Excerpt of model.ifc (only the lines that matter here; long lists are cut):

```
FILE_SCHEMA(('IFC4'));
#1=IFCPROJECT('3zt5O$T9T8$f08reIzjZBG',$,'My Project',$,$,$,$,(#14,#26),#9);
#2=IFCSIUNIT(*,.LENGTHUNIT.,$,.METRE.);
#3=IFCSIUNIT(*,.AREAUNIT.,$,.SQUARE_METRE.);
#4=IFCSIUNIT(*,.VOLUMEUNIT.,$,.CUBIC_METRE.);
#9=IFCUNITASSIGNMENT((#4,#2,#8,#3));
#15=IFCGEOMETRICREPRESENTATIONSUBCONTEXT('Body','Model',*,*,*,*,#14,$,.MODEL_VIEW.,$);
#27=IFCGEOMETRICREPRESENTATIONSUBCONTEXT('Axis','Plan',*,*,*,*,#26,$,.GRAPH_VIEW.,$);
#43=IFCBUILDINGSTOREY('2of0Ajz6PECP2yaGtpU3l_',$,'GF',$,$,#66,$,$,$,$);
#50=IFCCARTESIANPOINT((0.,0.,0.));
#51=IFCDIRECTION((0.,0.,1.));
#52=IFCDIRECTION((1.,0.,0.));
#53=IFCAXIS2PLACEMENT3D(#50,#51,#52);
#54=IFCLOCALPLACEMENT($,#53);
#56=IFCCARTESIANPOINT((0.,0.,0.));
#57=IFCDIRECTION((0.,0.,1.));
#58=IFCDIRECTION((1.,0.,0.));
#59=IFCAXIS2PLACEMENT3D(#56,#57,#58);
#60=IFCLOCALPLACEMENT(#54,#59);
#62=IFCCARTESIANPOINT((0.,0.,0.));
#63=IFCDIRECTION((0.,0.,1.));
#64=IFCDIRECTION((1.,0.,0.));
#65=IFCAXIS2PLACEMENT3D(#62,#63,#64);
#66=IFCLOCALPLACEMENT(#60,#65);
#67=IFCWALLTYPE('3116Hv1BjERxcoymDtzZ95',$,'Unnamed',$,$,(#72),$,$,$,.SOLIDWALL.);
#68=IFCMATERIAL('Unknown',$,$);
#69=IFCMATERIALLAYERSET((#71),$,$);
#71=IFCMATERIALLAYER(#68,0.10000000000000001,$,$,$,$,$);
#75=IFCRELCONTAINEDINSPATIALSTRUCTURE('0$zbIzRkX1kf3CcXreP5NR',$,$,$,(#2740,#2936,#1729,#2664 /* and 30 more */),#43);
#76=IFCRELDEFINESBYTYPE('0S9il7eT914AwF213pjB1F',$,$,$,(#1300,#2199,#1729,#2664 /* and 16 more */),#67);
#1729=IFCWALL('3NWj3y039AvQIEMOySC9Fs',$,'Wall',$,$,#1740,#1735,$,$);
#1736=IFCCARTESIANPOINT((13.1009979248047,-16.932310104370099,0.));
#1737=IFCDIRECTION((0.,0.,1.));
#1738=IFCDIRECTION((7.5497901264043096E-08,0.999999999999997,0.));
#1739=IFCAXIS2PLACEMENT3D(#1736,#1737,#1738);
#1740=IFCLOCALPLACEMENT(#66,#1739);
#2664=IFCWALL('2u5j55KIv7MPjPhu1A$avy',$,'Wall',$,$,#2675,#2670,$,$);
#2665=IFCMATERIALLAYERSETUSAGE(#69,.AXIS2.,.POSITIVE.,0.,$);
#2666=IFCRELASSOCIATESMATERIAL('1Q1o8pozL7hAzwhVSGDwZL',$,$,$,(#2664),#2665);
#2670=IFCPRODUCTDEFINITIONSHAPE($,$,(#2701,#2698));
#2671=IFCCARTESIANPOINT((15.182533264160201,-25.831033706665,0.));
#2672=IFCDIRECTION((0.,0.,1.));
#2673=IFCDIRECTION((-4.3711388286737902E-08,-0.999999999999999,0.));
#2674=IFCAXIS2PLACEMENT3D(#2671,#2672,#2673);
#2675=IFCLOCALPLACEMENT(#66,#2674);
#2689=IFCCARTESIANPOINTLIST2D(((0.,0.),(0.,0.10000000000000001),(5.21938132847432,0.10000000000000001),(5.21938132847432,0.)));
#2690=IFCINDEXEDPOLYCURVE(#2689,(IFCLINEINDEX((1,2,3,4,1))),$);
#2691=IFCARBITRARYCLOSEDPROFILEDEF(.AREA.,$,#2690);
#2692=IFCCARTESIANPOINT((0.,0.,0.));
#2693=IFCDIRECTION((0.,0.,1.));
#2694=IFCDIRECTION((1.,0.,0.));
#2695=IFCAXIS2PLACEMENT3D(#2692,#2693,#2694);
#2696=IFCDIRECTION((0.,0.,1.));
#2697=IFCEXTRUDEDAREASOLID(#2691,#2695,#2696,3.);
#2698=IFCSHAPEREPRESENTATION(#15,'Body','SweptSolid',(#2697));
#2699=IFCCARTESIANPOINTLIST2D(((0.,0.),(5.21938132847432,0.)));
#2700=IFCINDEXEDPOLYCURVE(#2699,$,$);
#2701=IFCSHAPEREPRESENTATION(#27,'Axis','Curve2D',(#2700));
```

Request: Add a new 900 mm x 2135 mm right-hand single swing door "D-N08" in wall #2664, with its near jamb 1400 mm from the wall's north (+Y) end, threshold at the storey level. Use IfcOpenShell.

```python
import numpy as np
import ifcopenshell
import ifcopenshell.api.feature
import ifcopenshell.api.geometry
import ifcopenshell.api.root
import ifcopenshell.api.spatial
import ifcopenshell.geom
import ifcopenshell.util.element
import ifcopenshell.util.placement
import ifcopenshell.util.representation
import ifcopenshell.util.shape
import ifcopenshell.util.unit

model = ifcopenshell.open("model.ifc")
unit_scale = ifcopenshell.util.unit.calculate_unit_scale(model)
settings = ifcopenshell.geom.settings()


def volume(element):
    """Net volume in cubic metres, openings subtracted."""
    shape = ifcopenshell.geom.create_shape(settings, element)
    return ifcopenshell.util.shape.get_volume(shape.geometry)


wall = model.by_guid("2u5j55KIv7MPjPhu1A$avy")
storey = ifcopenshell.util.element.get_container(wall, ifc_class="IfcBuildingStorey")
context = ifcopenshell.util.representation.get_context(model, "Model", "Body", "MODEL_VIEW")
before = volume(wall)

width, height, from_end, sill = 0.9, 2.135, 1.4, 0.0  # metres

# The wall runs along its own X axis, and the end named is its -X end.
wall_shape = ifcopenshell.geom.create_shape(settings, wall)
x, y, z = ifcopenshell.util.shape.get_vertices(wall_shape.geometry).T
start = x.min() + from_end
face, thickness = float(y.min()), float(y.max() - y.min())
wall_matrix = ifcopenshell.util.placement.get_local_placement(wall.ObjectPlacement)
level = ifcopenshell.util.placement.get_local_placement(storey.ObjectPlacement)[2, 3]


def in_wall(x, y):
    """Placement at x, y metres in the wall's axes, at sill height."""
    matrix = wall_matrix.copy()
    matrix[:, 3] = wall_matrix @ np.array([x / unit_scale, y / unit_scale, 0.0, 1.0])
    matrix[2, 3] = level + sill / unit_scale
    return matrix


# Opening: a box that overshoots both wall faces by 50 mm.
opening = ifcopenshell.api.root.create_entity(model, ifc_class="IfcOpeningElement", predefined_type="OPENING")
box = ifcopenshell.api.geometry.add_wall_representation(
    model, context=context, length=width, height=height, thickness=thickness + 0.1
)
ifcopenshell.api.geometry.assign_representation(model, product=opening, representation=box)
ifcopenshell.api.geometry.edit_object_placement(model, product=opening, matrix=in_wall(start, face - 0.05), is_si=False)
ifcopenshell.api.feature.add_feature(model, feature=opening, element=wall)

door = ifcopenshell.api.root.create_entity(model, ifc_class="IfcDoor", name="D-N08", predefined_type="DOOR")
door.OverallWidth, door.OverallHeight = width / unit_scale, height / unit_scale
door.OperationType = "SINGLE_SWING_RIGHT"
body = ifcopenshell.api.geometry.add_door_representation(
    model,
    context=context,
    overall_width=door.OverallWidth,
    overall_height=door.OverallHeight,
    operation_type="SINGLE_SWING_RIGHT",
    lining_properties={"LiningDepth": thickness / unit_scale, "ThresholdDepth": thickness / unit_scale},
)
ifcopenshell.api.geometry.assign_representation(model, product=door, representation=body)
ifcopenshell.api.spatial.assign_container(model, products=[door], relating_structure=storey)
ifcopenshell.api.feature.add_filling(model, opening=opening, element=door)

# The lining spans the wall, so the door starts at the wall face.
ifcopenshell.api.geometry.edit_object_placement(model, product=door, matrix=in_wall(start, face), is_si=False)

after = volume(wall)

print(f"wall volume {before:.3f} -> {after:.3f} m3")

model.write("model-out.ifc")
```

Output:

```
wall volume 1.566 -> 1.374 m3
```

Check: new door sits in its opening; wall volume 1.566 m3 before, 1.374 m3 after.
